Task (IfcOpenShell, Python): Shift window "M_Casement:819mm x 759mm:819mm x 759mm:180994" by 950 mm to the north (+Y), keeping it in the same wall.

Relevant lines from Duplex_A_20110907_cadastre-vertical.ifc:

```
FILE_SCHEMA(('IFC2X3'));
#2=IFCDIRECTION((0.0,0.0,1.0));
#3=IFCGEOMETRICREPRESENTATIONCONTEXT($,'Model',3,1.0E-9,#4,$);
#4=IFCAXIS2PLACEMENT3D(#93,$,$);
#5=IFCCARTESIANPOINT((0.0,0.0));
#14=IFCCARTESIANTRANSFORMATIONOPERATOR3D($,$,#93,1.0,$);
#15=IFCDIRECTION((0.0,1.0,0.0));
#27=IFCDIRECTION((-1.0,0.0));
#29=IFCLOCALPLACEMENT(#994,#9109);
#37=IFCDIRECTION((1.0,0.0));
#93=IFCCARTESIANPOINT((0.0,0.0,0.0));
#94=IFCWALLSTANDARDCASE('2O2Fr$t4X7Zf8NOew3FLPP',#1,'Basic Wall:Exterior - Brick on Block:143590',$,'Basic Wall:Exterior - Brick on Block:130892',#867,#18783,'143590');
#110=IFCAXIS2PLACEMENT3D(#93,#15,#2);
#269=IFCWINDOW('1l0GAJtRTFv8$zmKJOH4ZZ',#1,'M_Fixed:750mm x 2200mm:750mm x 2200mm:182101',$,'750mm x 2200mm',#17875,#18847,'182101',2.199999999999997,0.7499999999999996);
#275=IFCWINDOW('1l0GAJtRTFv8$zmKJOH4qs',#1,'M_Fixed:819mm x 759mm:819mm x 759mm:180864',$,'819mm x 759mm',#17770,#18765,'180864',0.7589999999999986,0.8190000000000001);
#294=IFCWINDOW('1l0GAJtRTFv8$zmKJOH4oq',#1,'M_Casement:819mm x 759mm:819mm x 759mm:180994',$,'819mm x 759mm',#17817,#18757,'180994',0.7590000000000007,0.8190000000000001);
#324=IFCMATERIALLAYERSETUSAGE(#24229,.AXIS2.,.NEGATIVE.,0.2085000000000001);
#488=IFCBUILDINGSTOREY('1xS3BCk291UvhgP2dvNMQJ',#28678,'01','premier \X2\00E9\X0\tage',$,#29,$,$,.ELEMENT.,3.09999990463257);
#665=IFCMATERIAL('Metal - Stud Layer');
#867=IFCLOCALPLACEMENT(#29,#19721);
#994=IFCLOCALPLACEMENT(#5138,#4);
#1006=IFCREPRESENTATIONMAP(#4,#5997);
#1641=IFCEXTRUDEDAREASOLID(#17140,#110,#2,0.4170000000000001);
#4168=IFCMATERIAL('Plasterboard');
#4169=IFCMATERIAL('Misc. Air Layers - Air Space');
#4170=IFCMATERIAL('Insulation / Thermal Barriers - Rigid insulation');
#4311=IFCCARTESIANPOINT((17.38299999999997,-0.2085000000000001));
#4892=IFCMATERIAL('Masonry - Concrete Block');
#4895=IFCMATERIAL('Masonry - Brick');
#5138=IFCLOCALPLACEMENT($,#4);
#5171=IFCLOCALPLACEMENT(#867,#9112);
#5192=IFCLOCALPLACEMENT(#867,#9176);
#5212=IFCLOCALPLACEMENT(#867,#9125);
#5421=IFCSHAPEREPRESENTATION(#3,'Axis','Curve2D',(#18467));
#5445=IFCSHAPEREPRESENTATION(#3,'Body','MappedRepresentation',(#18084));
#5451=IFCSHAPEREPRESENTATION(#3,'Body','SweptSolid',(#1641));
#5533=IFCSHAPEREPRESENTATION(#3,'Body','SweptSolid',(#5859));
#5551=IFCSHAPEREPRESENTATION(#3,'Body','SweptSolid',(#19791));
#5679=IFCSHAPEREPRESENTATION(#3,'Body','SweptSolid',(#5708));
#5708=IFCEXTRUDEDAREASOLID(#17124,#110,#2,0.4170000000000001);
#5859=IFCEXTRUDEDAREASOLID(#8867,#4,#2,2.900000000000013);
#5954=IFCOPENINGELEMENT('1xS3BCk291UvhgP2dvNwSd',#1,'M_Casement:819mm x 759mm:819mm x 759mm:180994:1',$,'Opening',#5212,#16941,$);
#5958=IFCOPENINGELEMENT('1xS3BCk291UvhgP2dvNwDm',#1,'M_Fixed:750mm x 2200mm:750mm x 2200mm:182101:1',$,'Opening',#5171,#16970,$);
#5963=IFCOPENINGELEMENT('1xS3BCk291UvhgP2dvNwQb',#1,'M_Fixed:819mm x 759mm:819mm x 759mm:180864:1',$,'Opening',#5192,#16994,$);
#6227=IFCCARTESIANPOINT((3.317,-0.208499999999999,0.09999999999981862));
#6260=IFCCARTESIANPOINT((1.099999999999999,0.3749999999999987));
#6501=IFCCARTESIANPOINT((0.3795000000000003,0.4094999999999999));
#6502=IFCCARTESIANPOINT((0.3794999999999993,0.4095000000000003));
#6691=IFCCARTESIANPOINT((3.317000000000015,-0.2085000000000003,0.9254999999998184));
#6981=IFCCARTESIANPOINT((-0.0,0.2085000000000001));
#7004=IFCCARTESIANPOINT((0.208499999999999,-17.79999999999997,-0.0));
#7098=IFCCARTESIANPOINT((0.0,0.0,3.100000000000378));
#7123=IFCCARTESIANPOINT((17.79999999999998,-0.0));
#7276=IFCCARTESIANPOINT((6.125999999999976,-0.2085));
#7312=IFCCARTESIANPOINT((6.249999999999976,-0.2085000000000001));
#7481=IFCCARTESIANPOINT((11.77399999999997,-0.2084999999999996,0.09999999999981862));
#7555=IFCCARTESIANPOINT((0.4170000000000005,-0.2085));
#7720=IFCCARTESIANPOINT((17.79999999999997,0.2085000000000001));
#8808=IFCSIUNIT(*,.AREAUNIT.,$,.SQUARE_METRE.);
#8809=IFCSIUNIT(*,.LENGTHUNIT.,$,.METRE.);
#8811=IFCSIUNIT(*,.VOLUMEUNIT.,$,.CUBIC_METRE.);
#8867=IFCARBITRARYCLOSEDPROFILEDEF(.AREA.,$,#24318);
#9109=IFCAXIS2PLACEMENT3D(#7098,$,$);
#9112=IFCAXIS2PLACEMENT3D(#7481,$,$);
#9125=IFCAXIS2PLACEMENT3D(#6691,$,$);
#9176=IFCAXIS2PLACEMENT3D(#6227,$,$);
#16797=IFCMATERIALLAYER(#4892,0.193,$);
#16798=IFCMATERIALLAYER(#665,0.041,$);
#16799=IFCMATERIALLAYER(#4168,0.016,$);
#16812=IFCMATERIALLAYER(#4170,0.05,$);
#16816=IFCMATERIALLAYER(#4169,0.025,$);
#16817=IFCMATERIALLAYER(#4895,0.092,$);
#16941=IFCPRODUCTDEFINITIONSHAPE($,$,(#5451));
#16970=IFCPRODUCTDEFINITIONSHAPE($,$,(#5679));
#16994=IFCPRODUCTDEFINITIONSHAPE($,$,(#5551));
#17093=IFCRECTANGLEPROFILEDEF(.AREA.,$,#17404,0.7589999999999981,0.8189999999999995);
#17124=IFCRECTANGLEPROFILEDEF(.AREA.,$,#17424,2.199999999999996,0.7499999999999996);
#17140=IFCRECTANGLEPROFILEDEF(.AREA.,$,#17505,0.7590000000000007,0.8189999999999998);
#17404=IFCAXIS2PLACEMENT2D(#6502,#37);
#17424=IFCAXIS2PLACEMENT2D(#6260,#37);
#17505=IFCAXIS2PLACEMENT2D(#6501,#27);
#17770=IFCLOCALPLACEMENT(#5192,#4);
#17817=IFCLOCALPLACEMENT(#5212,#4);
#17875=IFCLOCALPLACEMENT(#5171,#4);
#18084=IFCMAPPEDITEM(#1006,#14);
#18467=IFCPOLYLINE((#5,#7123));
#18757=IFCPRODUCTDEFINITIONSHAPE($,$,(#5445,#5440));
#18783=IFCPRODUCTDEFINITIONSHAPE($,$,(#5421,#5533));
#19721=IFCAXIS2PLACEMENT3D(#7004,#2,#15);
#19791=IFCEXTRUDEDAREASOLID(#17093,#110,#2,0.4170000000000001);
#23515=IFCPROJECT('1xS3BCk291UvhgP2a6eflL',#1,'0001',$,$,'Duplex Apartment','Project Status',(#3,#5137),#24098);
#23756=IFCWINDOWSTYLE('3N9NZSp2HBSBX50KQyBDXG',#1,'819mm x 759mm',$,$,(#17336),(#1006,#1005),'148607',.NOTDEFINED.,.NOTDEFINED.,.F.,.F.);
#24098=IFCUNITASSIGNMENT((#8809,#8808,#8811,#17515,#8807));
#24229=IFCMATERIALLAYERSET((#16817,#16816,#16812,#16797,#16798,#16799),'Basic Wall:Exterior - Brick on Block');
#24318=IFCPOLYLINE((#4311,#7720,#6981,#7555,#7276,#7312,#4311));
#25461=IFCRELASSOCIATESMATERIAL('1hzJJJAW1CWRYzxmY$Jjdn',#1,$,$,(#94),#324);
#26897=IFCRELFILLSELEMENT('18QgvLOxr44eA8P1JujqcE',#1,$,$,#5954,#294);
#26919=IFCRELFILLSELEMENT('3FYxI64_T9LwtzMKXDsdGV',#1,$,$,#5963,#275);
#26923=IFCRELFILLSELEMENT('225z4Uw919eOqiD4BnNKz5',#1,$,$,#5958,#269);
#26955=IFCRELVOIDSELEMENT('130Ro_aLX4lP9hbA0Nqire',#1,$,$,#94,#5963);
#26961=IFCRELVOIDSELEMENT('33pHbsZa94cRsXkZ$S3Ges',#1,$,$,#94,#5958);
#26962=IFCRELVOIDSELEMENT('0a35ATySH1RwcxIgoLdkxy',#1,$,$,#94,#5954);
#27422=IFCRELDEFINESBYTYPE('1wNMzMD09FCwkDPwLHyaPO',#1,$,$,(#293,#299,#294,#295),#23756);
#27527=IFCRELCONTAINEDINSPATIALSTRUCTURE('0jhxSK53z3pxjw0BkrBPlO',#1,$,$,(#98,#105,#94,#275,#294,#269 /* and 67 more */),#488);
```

```python
import ifcopenshell
import ifcopenshell.api.geometry
import ifcopenshell.util.placement
import ifcopenshell.util.unit

model = ifcopenshell.open("Duplex_A_20110907_cadastre-vertical.ifc")
unit_scale = ifcopenshell.util.unit.calculate_unit_scale(model)

window = model.by_guid("1l0GAJtRTFv8$zmKJOH4oq")
opening = window.FillsVoids[0].RelatingOpeningElement
wall = opening.VoidsElements[0].RelatingBuildingElement

wall_matrix = ifcopenshell.util.placement.get_local_placement(wall.ObjectPlacement)
shift = wall_matrix[:3, 0] * 0.95 / unit_scale
before = ifcopenshell.util.placement.get_local_placement(window.ObjectPlacement)[:3, 3].copy()

# The window is placed relative to its opening, so it follows when the opening moves.
matrix = ifcopenshell.util.placement.get_local_placement(opening.ObjectPlacement)
matrix[:3, 3] += shift
ifcopenshell.api.geometry.edit_object_placement(
    model, product=opening, matrix=matrix, is_si=False, should_transform_children=True
)

after = ifcopenshell.util.placement.get_local_placement(window.ObjectPlacement)[:3, 3]
print("window moved by", (after - before).round(3) + 0.0)

model.write("Duplex_A_20110907_cadastre-vertical-out.ifc")
```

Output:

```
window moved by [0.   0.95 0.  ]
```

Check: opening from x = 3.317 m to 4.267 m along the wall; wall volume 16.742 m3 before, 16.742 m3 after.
